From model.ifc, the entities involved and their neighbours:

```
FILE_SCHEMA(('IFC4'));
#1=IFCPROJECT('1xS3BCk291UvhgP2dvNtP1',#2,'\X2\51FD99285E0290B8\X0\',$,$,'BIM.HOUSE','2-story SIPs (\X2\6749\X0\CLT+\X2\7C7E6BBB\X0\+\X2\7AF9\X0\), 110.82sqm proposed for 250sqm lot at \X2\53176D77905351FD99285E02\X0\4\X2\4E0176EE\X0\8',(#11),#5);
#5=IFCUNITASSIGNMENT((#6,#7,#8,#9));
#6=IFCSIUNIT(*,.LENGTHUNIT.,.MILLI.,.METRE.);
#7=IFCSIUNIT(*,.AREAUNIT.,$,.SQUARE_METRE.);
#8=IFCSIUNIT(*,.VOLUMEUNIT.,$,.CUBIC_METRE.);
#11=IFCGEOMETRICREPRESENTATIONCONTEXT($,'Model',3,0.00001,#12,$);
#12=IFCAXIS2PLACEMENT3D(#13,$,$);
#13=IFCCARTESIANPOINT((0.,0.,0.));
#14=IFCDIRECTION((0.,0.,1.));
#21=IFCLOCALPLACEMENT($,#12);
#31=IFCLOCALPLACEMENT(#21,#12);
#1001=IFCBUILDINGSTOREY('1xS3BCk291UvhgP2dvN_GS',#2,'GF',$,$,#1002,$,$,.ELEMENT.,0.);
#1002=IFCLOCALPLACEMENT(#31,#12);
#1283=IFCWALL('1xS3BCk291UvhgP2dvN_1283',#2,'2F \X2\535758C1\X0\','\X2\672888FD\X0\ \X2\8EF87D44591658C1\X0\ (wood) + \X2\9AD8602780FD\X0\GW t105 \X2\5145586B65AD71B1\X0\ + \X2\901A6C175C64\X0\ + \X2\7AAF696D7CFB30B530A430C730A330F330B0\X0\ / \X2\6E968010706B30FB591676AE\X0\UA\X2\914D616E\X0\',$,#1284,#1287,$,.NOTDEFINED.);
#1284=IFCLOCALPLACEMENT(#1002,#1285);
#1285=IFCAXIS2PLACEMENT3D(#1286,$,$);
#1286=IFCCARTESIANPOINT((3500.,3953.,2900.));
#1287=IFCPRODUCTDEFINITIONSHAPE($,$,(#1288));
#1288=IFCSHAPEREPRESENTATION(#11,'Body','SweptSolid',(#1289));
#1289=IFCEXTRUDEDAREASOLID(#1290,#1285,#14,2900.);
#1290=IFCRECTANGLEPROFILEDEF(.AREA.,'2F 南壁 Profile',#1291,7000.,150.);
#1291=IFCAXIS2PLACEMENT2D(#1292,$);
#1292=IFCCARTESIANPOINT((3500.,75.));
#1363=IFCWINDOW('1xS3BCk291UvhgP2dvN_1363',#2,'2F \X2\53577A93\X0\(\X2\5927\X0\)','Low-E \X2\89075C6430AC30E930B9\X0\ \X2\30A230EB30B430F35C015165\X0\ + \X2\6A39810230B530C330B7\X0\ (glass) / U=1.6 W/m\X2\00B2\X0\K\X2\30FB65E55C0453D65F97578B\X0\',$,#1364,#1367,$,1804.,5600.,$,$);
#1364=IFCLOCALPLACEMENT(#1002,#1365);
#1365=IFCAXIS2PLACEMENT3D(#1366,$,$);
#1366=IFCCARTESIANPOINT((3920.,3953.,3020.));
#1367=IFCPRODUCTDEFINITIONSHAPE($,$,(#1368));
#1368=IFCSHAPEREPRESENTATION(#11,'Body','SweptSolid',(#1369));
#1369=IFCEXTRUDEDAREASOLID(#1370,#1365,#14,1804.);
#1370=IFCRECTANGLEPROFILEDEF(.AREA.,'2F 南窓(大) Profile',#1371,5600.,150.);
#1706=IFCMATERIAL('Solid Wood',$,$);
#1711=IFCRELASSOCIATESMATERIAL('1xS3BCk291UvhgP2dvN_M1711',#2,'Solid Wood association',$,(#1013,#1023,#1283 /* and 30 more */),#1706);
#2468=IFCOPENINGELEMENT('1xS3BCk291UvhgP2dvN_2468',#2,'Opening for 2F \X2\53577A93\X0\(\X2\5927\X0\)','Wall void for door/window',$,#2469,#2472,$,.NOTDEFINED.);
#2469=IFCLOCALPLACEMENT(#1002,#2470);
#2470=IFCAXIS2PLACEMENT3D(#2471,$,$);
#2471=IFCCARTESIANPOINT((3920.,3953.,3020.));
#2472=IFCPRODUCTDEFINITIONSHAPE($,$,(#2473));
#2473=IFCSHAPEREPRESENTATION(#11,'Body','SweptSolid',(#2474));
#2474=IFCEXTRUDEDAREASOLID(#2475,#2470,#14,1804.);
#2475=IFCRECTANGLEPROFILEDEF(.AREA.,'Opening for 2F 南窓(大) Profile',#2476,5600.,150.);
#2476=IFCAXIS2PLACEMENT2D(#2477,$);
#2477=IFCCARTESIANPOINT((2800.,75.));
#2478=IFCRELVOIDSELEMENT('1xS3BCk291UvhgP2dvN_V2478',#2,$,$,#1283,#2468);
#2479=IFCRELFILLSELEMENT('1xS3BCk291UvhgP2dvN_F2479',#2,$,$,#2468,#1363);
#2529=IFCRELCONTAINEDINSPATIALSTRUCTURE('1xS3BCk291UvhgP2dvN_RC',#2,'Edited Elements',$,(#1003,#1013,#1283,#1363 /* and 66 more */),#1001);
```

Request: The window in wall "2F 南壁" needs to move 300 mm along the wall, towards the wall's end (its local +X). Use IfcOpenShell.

```python
import ifcopenshell
import ifcopenshell.api.geometry
import ifcopenshell.util.placement
import ifcopenshell.util.unit

model = ifcopenshell.open("model.ifc")
unit_scale = ifcopenshell.util.unit.calculate_unit_scale(model)

window = model.by_id(1363)
opening = window.FillsVoids[0].RelatingOpeningElement
wall = opening.VoidsElements[0].RelatingBuildingElement

wall_matrix = ifcopenshell.util.placement.get_local_placement(wall.ObjectPlacement)
shift = wall_matrix[:3, 0] * 0.3 / unit_scale
before = ifcopenshell.util.placement.get_local_placement(window.ObjectPlacement)[:3, 3].copy()

# The window is not placed relative to its opening, so move both.
for product in (opening, window):
    matrix = ifcopenshell.util.placement.get_local_placement(product.ObjectPlacement)
    matrix[:3, 3] += shift
    ifcopenshell.api.geometry.edit_object_placement(model, product=product, matrix=matrix, is_si=False)

after = ifcopenshell.util.placement.get_local_placement(window.ObjectPlacement)[:3, 3]
print("window moved by", (after - before).round(3) + 0.0)

model.write("model_rev.ifc")
```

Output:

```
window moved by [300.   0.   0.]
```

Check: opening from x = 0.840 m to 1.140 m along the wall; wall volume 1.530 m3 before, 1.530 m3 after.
